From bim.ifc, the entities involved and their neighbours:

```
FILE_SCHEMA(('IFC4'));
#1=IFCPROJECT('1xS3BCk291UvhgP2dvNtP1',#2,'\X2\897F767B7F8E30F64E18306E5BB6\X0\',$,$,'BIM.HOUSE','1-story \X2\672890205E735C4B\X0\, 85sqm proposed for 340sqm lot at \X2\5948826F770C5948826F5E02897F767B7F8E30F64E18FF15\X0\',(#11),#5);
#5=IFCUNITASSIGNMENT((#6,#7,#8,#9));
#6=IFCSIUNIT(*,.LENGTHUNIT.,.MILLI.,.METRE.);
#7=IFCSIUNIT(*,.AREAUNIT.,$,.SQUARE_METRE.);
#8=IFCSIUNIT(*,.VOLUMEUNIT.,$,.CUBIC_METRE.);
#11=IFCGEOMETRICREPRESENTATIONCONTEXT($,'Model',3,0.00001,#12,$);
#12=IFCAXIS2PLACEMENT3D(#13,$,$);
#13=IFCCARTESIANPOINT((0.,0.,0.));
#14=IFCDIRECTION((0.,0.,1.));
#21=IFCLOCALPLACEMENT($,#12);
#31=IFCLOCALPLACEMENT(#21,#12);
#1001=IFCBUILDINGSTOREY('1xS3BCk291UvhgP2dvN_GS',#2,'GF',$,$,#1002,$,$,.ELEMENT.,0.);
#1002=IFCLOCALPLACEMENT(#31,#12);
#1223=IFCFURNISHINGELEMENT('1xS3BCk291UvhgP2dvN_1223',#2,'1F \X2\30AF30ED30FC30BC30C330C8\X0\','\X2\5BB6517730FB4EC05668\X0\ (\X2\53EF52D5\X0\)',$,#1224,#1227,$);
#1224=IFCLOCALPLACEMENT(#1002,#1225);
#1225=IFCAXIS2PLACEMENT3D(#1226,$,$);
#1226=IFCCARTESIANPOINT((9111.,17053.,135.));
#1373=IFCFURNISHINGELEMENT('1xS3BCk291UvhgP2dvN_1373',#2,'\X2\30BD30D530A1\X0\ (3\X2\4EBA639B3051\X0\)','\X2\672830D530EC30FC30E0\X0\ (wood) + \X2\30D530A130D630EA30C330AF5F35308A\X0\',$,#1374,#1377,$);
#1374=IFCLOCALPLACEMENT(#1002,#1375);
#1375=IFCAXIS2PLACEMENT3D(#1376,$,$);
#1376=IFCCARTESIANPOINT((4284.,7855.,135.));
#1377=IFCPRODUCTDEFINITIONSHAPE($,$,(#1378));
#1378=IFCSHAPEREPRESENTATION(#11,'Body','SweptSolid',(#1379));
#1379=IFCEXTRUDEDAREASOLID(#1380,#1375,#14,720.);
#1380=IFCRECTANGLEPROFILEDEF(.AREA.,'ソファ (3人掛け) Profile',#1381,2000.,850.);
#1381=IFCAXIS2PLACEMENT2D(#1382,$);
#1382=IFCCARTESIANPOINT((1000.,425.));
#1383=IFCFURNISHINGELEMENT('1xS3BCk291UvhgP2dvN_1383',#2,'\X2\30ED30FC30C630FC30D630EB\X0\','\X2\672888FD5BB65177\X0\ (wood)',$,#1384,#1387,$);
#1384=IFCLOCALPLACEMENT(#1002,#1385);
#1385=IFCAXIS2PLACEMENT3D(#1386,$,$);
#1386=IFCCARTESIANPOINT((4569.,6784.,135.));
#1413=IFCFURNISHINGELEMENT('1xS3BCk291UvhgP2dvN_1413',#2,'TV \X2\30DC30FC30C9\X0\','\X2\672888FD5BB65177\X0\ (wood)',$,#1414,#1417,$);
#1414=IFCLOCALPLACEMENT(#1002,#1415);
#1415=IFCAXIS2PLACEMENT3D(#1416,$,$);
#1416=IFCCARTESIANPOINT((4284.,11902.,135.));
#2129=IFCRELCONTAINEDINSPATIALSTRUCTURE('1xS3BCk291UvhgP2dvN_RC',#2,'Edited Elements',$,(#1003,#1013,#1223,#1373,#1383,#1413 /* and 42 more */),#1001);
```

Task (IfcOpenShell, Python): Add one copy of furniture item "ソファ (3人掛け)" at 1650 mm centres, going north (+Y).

```python
import numpy as np
import ifcopenshell
import ifcopenshell.api.geometry
import ifcopenshell.api.root
import ifcopenshell.util.element
import ifcopenshell.util.placement

model = ifcopenshell.open("bim.ifc")


def reuse_history(source, copy):
    """copy_class also copies each property set's owner history, people and application; keep the originals."""
    for rel in copy.IsDefinedBy:
        if rel.is_a("IfcRelDefinesByProperties") and (history := rel.RelatingPropertyDefinition.OwnerHistory):
            rel.RelatingPropertyDefinition.OwnerHistory = source.OwnerHistory
            ifcopenshell.util.element.remove_deep2(model, history)


source = model.by_guid("1xS3BCk291UvhgP2dvN_1373")
base = ifcopenshell.util.placement.get_local_placement(source.ObjectPlacement)
step = np.array([0.0, 1.0, 0.0]) * 1650.0

for i in range(1, 2):
    copy = ifcopenshell.api.root.copy_class(model, product=source)
    copy.Representation = ifcopenshell.util.element.copy_deep(
        model, source.Representation, exclude=["IfcGeometricRepresentationContext", "IfcRepresentationMap"]
    )
    reuse_history(source, copy)
    matrix = base.copy()
    matrix[:3, 3] += i * step
    print("added at", matrix[:3, 3].round(3) + 0.0)
    ifcopenshell.api.geometry.edit_object_placement(model, product=copy, matrix=matrix, is_si=False)

model.write("bim_v2.ifc")
```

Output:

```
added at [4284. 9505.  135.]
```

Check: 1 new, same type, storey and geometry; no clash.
